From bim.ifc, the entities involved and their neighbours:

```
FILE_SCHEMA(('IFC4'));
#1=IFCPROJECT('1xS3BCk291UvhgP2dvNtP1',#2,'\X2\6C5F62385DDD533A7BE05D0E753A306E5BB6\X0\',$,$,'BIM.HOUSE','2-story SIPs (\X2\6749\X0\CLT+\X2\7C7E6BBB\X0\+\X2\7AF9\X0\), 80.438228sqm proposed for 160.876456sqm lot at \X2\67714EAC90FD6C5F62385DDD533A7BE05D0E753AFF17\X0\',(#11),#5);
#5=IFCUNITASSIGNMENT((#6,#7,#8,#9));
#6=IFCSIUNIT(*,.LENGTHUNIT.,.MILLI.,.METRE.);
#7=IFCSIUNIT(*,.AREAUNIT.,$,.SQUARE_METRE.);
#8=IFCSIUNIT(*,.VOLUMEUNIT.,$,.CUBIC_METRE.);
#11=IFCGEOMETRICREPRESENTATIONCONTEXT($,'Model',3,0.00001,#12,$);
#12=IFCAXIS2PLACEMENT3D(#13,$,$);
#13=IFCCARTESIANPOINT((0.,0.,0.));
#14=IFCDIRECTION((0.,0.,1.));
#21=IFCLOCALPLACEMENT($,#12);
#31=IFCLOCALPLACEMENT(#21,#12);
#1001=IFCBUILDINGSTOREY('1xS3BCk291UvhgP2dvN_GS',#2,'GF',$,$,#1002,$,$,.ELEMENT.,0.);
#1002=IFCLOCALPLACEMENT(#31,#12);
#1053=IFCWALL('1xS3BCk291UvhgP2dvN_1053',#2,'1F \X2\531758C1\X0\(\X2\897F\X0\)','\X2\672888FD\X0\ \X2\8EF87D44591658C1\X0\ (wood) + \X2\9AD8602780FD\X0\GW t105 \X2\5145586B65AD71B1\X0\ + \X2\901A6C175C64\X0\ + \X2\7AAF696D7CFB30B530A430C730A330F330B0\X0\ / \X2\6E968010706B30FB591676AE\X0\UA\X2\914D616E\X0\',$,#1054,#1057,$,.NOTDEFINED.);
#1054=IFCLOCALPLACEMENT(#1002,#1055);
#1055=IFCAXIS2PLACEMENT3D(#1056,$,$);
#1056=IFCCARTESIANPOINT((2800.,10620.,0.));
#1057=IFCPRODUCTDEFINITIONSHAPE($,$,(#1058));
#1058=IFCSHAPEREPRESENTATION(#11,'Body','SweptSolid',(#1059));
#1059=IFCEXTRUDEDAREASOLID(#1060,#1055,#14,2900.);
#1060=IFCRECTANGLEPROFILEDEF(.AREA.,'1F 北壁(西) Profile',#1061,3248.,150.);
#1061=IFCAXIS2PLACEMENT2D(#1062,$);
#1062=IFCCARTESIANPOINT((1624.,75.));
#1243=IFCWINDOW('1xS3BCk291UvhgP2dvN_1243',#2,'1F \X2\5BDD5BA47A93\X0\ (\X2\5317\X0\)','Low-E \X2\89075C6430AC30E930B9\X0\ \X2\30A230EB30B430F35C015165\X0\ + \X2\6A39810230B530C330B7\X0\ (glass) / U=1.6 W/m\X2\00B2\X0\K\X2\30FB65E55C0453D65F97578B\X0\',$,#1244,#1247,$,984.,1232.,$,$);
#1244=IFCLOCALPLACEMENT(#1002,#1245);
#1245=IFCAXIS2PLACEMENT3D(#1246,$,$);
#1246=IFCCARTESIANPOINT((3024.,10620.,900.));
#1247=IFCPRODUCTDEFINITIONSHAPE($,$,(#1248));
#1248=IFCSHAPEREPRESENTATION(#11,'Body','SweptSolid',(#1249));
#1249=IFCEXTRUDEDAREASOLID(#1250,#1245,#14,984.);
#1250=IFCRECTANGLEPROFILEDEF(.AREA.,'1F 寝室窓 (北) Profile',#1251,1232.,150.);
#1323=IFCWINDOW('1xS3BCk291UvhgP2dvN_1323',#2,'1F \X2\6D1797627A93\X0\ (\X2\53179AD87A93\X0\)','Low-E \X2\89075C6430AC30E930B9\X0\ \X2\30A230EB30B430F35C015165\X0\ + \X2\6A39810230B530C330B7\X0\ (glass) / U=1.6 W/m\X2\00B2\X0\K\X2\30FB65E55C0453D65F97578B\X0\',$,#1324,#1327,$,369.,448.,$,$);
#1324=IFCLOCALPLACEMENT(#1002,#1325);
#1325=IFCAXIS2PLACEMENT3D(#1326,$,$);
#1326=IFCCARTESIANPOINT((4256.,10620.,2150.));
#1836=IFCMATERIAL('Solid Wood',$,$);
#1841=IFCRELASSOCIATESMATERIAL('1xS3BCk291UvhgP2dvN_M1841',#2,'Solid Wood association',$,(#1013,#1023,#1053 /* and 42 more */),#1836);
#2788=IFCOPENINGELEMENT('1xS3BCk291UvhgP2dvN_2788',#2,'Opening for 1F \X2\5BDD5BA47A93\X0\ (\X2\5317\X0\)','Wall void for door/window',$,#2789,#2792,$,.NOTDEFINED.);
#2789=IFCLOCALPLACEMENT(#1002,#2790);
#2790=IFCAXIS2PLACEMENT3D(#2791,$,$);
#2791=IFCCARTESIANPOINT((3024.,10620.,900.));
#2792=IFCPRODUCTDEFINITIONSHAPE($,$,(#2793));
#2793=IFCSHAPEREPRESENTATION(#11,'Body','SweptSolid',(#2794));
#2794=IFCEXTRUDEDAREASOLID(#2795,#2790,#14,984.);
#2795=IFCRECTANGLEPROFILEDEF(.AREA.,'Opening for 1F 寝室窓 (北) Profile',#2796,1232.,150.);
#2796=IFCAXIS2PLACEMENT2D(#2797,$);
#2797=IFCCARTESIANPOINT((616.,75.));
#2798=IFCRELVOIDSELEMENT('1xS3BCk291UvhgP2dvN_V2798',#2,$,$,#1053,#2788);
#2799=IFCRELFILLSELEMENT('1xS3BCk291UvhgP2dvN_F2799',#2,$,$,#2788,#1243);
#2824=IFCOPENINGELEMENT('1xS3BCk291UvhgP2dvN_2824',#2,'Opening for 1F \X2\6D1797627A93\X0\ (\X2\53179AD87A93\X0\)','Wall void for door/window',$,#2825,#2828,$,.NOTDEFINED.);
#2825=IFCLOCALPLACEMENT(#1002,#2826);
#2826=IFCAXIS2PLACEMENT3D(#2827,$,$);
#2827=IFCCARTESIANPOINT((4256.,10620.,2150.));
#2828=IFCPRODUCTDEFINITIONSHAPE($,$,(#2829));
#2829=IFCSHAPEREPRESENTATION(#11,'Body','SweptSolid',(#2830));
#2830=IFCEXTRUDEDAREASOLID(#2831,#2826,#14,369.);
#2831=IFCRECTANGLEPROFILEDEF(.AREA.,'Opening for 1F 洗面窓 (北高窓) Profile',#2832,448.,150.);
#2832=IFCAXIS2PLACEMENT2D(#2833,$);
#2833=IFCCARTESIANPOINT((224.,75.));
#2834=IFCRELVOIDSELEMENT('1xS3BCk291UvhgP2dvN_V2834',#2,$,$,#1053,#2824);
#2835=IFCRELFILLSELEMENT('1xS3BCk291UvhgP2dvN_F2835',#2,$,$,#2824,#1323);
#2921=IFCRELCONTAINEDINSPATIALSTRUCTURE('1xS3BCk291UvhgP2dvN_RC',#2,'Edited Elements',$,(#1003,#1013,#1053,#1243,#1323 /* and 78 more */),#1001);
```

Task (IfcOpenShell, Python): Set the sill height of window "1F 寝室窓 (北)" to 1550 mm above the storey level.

```python
import numpy as np
import ifcopenshell
import ifcopenshell.api.geometry
import ifcopenshell.geom
import ifcopenshell.util.element
import ifcopenshell.util.placement
import ifcopenshell.util.shape
import ifcopenshell.util.unit

model = ifcopenshell.open("bim.ifc")
unit_scale = ifcopenshell.util.unit.calculate_unit_scale(model)

window = model.by_guid("1xS3BCk291UvhgP2dvN_1243")
opening = window.FillsVoids[0].RelatingOpeningElement
storey = ifcopenshell.util.element.get_container(window, ifc_class="IfcBuildingStorey")
level = ifcopenshell.util.placement.get_local_placement(storey.ObjectPlacement)[2, 3]

# The opening's origin need not be at the sill, so measure its lowest point.
shape = ifcopenshell.geom.create_shape(ifcopenshell.geom.settings(), opening)
bottom = ifcopenshell.util.shape.get_shape_bottom_elevation(shape, shape.geometry) / unit_scale
dz = level + 1.55 / unit_scale - bottom

shift = np.array([0.0, 0.0, dz])
# The window is not placed relative to its opening, so move both.
for product in (opening, window):
    matrix = ifcopenshell.util.placement.get_local_placement(product.ObjectPlacement)
    matrix[:3, 3] += shift
    ifcopenshell.api.geometry.edit_object_placement(model, product=product, matrix=matrix, is_si=False)

print(f"moved by {dz * unit_scale:+.3f} m")

model.write("bim_edited.ifc")
```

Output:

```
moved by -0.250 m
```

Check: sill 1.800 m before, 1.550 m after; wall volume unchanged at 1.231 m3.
